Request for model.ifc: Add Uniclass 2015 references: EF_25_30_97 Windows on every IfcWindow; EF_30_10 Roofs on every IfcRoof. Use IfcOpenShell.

First a look at what the model holds.

```python
import ifcopenshell

model = ifcopenshell.open("model.ifc")
print(model.schema)
print("classifications:", [c.Name for c in model.by_type("IfcClassification")])
for ifc_class in ("IfcDoor", "IfcRoof", "IfcStair", "IfcWall", "IfcWindow"):
    print(ifc_class, len(model.by_type(ifc_class)))
```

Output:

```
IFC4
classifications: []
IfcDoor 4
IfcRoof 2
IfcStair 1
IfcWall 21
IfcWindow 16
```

```python
import ifcopenshell
import ifcopenshell.api.classification

model = ifcopenshell.open("model.ifc")

system = ifcopenshell.api.classification.add_classification(model, classification="Uniclass 2015")

codes = {
    "IfcWindow": ("EF_25_30_97", "Windows"),
    "IfcRoof": ("EF_30_10", "Roofs"),
}
for ifc_class, (code, name) in codes.items():
    products = model.by_type(ifc_class)
    ifcopenshell.api.classification.add_reference(
        model, products=products, classification=system, identification=code, name=name
    )
    print(code, len(products))

model.write("model_v2.ifc")
```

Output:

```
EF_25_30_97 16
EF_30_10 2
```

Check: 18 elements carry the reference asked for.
